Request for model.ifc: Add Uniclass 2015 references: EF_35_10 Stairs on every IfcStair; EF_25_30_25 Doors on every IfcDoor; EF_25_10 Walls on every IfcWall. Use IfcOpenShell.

First a look at what the model holds.

```python
import ifcopenshell

model = ifcopenshell.open("model.ifc")
print(model.schema)
print("classifications:", [c.Name for c in model.by_type("IfcClassification")])
for ifc_class in ("IfcDoor", "IfcRoof", "IfcStair", "IfcWall", "IfcWindow"):
    print(ifc_class, len(model.by_type(ifc_class)))
```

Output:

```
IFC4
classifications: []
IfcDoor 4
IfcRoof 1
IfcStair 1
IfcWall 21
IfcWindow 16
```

```python
import ifcopenshell
import ifcopenshell.api.classification

model = ifcopenshell.open("model.ifc")

system = ifcopenshell.api.classification.add_classification(model, classification="Uniclass 2015")

codes = {
    "IfcStair": ("EF_35_10", "Stairs"),
    "IfcDoor": ("EF_25_30_25", "Doors"),
    "IfcWall": ("EF_25_10", "Walls"),
}
for ifc_class, (code, name) in codes.items():
    products = model.by_type(ifc_class)
    ifcopenshell.api.classification.add_reference(
        model, products=products, classification=system, identification=code, name=name
    )
    print(code, len(products))

model.write("model_edited.ifc")
```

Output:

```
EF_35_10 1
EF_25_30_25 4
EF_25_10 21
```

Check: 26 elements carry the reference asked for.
